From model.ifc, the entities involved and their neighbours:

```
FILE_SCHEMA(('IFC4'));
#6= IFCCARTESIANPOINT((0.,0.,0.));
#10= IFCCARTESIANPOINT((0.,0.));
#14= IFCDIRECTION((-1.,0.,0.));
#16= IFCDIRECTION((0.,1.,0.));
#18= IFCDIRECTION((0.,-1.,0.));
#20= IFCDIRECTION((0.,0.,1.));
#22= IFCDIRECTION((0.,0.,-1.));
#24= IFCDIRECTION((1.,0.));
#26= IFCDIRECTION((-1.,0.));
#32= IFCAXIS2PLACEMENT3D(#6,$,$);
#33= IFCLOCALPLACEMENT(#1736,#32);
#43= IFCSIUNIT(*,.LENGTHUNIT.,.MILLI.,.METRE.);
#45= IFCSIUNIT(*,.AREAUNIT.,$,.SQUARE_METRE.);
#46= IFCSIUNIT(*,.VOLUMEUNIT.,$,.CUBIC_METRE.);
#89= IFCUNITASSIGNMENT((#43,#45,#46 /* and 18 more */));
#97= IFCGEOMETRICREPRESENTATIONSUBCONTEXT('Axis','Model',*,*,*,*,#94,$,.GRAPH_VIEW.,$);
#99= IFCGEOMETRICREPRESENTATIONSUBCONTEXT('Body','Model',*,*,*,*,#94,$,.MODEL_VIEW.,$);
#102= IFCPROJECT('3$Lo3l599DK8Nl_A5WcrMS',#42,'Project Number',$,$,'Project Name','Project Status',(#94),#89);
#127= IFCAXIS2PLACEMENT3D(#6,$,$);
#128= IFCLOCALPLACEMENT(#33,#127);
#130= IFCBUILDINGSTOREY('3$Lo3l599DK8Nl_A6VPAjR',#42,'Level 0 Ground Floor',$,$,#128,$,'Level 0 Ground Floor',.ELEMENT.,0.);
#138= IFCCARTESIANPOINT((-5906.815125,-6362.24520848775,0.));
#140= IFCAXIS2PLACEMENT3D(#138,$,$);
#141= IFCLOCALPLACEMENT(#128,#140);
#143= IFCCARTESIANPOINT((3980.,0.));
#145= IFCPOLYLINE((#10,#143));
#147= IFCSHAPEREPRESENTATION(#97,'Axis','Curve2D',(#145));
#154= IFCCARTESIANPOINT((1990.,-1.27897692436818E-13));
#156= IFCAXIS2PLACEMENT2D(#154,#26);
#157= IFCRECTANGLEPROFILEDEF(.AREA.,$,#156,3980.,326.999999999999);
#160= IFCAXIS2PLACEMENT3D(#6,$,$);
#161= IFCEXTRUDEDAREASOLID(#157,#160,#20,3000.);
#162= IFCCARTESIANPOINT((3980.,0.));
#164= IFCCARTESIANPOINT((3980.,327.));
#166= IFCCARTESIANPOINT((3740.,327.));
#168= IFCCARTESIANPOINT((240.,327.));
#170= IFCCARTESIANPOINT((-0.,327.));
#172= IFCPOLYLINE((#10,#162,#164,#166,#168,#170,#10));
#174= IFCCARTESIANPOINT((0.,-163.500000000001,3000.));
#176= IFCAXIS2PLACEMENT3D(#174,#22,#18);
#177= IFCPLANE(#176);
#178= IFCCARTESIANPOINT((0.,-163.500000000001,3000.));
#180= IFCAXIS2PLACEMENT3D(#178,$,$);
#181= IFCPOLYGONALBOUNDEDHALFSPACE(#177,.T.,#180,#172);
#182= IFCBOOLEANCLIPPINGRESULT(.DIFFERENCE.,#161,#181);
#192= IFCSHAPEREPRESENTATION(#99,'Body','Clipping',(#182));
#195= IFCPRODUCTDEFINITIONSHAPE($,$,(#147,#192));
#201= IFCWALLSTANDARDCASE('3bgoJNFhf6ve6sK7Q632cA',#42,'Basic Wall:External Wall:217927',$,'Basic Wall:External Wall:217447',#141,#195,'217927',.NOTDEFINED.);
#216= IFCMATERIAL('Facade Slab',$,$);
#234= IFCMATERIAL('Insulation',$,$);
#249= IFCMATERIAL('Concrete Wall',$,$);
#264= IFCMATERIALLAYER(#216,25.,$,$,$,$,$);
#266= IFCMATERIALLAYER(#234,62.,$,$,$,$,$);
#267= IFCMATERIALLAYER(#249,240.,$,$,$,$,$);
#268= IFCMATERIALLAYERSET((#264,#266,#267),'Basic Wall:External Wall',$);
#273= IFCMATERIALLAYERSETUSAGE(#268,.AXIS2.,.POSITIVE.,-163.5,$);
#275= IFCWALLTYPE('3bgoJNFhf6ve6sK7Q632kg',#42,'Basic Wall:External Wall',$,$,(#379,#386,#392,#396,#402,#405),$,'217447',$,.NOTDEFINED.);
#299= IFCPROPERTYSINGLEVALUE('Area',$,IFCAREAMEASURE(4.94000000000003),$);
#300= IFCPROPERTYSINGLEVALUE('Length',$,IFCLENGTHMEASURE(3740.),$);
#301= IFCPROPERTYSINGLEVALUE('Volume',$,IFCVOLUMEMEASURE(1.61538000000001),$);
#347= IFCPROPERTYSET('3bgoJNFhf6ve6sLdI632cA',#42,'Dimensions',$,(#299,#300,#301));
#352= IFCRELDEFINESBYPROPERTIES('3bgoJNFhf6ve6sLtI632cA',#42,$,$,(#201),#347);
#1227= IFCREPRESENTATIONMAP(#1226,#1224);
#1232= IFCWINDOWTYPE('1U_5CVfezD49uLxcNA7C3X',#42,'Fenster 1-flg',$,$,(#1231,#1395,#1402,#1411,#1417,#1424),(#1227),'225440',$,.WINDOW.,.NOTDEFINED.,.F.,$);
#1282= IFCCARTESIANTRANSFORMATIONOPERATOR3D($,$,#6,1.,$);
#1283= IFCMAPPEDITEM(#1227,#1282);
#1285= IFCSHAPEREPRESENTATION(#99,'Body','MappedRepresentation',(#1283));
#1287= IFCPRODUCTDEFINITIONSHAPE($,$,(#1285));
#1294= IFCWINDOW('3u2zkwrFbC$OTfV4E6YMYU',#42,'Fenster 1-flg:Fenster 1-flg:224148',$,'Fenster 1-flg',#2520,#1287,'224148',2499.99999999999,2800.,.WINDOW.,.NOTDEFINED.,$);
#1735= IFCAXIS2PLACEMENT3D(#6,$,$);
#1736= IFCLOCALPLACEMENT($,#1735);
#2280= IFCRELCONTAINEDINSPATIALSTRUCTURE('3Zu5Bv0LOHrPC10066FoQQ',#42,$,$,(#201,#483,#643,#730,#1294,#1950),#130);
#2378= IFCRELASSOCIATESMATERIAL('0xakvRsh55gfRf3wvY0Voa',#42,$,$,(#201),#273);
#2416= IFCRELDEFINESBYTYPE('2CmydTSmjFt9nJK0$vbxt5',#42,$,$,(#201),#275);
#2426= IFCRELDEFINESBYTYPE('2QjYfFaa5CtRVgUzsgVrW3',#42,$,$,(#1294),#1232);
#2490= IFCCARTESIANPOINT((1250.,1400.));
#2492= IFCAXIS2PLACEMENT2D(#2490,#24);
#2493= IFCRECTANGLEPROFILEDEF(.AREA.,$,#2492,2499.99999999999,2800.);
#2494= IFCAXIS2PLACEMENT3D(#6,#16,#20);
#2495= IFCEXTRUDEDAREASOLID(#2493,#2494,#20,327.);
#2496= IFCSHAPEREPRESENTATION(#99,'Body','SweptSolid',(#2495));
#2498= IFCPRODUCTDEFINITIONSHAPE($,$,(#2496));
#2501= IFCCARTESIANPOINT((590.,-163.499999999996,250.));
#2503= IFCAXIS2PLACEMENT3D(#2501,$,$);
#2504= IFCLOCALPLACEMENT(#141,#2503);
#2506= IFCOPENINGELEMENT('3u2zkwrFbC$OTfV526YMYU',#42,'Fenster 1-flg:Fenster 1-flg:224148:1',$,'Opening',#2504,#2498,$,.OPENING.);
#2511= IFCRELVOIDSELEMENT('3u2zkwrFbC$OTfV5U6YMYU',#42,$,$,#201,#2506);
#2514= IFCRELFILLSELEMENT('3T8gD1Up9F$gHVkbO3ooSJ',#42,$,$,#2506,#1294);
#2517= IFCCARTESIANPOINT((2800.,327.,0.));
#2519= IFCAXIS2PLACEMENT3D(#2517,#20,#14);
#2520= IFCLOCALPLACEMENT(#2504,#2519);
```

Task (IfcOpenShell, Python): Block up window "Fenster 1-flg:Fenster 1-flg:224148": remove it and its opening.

```python
import ifcopenshell
import ifcopenshell.api.feature
import ifcopenshell.api.pset
import ifcopenshell.api.root
import ifcopenshell.geom
import ifcopenshell.util.element
import ifcopenshell.util.shape
import ifcopenshell.util.unit

model = ifcopenshell.open("model.ifc")
area_scale = ifcopenshell.util.unit.calculate_unit_scale(model, "AREAUNIT")
volume_scale = ifcopenshell.util.unit.calculate_unit_scale(model, "VOLUMEUNIT")
settings = ifcopenshell.geom.settings()


def volume(element):
    """Net volume in cubic metres, openings subtracted."""
    shape = ifcopenshell.geom.create_shape(settings, element)
    return ifcopenshell.util.shape.get_volume(shape.geometry)


window = model.by_guid("3u2zkwrFbC$OTfV4E6YMYU")
opening = window.FillsVoids[0].RelatingOpeningElement
wall = opening.VoidsElements[0].RelatingBuildingElement
before = volume(wall)

ifcopenshell.api.root.remove_product(model, product=window)
ifcopenshell.api.feature.remove_feature(model, feature=opening)

after = volume(wall)
thickness = 0.327  # wall thickness in metres

# Update the wall's stored quantities.
pset = model.by_id(ifcopenshell.util.element.get_pset(wall, "Dimensions", should_inherit=False)["id"])
ifcopenshell.api.pset.edit_pset(model, pset=pset, properties={
    "Area": model.create_entity("IfcAreaMeasure", after / thickness / area_scale),
    "Volume": model.create_entity("IfcVolumeMeasure", after / volume_scale),
})

print(f"wall volume {before:.3f} -> {after:.3f} m3")

model.write("model_rev.ifc")
```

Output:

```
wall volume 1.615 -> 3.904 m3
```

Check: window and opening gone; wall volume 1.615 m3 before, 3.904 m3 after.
